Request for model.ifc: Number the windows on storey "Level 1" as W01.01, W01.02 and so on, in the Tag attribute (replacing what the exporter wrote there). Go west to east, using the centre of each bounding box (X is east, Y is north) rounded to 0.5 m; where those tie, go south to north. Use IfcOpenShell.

First a look at what the model holds.

```python
import ifcopenshell
import ifcopenshell.util.element
import ifcopenshell.util.placement

model = ifcopenshell.open("model.ifc")
print(model.schema)
storey = next(s for s in model.by_type("IfcBuildingStorey") if s.Name == "Level 1")
windows = [e for e in ifcopenshell.util.element.get_decomposition(storey) if e.is_a("IfcWindow")]
for e in sorted(windows, key=lambda e: e.id()):
    origin = ifcopenshell.util.placement.get_local_placement(e.ObjectPlacement)[:3, 3]
    print(e.id(), e.Tag, e.Name, origin.round(2) + 0.0, sep=" | ")
```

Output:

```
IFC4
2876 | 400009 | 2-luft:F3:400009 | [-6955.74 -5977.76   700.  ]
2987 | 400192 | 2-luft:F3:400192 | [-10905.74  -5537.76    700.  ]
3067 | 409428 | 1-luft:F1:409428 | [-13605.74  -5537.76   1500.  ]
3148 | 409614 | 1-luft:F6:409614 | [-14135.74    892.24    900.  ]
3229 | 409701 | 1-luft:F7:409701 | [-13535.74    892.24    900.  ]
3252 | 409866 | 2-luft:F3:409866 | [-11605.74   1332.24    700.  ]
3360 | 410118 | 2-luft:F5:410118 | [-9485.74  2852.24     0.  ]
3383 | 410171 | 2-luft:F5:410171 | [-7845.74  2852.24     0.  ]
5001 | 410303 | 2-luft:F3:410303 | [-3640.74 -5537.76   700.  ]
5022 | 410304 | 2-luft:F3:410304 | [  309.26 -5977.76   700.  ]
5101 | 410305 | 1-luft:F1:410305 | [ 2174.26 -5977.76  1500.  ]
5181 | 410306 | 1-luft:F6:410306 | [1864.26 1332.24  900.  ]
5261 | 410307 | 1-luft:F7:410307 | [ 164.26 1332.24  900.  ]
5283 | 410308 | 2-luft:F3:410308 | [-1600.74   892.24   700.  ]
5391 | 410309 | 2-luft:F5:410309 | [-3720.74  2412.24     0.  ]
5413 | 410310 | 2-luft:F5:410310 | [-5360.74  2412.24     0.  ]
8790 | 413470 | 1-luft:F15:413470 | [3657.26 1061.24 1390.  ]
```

```python
import ifcopenshell
import ifcopenshell.geom
import ifcopenshell.util.element
import ifcopenshell.util.shape

model = ifcopenshell.open("model.ifc")
settings = ifcopenshell.geom.settings()
settings.set("use-world-coords", True)


def centre(element):
    shape = ifcopenshell.geom.create_shape(settings, element)
    return ifcopenshell.util.shape.get_bbox_centroid(shape.geometry)


storey = next(s for s in model.by_type("IfcBuildingStorey") if s.Name == "Level 1")
windows = [e for e in ifcopenshell.util.element.get_decomposition(storey) if e.is_a("IfcWindow")]

# Insertion points can sit at a corner or the storey origin, so sort by the geometry (in metres).
centres = {e: centre(e) for e in windows}
windows.sort(key=lambda e: (round(centres[e][0] / 0.5), centres[e][1]))

for i, e in enumerate(windows, start=1):
    number = f"W01.{i:02d}"
    e.Tag = number
    print(e.id(), number)

model.write("model_v2.ifc")
```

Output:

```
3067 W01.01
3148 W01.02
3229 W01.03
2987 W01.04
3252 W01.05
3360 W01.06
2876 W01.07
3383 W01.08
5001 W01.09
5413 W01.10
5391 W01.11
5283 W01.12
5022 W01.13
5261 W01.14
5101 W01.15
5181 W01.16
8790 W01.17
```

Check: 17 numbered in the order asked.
